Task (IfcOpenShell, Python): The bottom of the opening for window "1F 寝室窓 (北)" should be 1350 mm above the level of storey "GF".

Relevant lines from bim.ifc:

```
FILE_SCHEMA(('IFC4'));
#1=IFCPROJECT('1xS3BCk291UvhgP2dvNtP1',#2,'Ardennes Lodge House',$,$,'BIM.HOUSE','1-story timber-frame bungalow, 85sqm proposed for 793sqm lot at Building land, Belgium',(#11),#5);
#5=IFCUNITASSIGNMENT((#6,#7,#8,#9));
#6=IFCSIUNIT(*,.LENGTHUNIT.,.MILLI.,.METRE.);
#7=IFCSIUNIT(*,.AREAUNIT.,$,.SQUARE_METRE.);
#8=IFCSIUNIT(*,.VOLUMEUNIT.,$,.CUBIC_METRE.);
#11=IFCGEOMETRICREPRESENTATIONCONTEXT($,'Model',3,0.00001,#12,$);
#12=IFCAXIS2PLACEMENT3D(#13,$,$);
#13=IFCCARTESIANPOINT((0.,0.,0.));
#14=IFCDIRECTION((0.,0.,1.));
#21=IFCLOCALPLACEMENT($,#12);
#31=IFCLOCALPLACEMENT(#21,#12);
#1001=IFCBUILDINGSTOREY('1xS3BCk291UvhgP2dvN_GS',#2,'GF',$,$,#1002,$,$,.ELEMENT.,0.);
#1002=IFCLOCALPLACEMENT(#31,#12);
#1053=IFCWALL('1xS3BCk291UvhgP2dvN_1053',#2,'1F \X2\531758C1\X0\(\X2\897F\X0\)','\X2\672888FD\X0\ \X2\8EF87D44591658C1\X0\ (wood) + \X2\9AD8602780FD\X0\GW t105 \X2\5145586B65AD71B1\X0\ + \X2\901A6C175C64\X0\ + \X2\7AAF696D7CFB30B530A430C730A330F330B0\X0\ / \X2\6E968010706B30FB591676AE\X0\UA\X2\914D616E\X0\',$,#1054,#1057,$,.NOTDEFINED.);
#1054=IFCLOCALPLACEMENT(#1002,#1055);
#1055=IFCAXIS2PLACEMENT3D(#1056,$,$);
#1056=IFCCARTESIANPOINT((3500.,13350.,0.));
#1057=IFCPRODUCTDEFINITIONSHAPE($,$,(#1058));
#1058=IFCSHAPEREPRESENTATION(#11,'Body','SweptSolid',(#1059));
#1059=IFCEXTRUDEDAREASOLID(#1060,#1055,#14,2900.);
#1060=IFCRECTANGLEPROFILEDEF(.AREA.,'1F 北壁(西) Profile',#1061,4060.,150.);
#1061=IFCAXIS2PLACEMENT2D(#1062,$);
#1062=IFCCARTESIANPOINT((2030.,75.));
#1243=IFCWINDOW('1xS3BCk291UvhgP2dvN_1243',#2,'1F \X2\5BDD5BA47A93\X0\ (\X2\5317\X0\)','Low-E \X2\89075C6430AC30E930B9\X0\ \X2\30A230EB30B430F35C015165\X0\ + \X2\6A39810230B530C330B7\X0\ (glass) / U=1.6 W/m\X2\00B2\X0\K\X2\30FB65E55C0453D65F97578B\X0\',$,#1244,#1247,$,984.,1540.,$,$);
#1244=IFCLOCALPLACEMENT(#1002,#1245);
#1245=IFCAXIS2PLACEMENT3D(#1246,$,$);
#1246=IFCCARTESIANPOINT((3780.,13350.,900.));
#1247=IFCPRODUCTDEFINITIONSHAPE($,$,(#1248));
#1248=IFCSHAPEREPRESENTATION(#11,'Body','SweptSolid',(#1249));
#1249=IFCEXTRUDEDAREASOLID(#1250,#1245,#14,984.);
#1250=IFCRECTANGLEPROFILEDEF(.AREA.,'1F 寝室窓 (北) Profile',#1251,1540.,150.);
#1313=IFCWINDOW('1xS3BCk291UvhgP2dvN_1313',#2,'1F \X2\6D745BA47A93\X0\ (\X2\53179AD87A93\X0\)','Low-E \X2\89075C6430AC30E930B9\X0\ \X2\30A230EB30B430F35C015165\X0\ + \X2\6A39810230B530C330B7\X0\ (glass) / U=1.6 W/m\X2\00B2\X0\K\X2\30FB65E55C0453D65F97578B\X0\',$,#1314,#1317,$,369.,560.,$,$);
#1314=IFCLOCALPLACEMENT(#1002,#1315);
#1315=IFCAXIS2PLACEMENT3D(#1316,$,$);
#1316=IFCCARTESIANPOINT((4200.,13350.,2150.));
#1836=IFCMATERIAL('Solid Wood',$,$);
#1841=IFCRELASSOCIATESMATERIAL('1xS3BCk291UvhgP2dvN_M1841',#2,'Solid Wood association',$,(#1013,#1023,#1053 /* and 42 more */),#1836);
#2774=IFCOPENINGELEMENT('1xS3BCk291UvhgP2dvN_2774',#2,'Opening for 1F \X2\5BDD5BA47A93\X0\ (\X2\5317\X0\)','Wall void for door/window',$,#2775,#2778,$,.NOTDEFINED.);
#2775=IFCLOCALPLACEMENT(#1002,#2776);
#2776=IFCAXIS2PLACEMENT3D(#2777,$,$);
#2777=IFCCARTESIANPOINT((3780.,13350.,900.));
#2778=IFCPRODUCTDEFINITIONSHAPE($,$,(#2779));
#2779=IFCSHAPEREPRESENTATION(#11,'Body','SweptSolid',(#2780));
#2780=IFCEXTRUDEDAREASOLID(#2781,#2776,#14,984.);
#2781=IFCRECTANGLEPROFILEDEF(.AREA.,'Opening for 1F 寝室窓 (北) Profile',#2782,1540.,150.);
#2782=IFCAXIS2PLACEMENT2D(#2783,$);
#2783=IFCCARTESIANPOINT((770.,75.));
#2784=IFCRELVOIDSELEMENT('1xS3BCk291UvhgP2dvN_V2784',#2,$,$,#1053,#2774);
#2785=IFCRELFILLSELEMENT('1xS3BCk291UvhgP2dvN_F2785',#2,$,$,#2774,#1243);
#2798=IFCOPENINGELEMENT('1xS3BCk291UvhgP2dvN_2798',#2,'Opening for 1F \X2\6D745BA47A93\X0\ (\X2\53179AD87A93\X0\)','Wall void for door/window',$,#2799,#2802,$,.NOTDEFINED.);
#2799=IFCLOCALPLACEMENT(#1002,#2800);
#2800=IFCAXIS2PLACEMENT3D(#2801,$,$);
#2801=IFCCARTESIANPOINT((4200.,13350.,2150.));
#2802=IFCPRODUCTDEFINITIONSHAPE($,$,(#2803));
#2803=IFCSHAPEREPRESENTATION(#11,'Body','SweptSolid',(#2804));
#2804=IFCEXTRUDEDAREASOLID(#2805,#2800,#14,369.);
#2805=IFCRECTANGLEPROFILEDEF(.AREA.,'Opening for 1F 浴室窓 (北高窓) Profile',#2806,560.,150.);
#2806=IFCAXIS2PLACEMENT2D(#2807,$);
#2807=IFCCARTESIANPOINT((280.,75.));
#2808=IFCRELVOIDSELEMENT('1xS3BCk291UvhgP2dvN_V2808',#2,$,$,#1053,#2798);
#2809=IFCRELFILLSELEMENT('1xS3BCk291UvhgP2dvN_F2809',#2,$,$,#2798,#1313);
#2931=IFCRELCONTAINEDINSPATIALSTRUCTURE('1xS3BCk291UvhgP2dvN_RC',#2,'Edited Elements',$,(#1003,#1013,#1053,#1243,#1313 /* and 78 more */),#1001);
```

```python
import numpy as np
import ifcopenshell
import ifcopenshell.api.geometry
import ifcopenshell.geom
import ifcopenshell.util.element
import ifcopenshell.util.placement
import ifcopenshell.util.shape
import ifcopenshell.util.unit

model = ifcopenshell.open("bim.ifc")
unit_scale = ifcopenshell.util.unit.calculate_unit_scale(model)

window = model.by_guid("1xS3BCk291UvhgP2dvN_1243")
opening = window.FillsVoids[0].RelatingOpeningElement
storey = ifcopenshell.util.element.get_container(window, ifc_class="IfcBuildingStorey")
level = ifcopenshell.util.placement.get_local_placement(storey.ObjectPlacement)[2, 3]

# The opening's origin need not be at the sill, so measure its lowest point.
shape = ifcopenshell.geom.create_shape(ifcopenshell.geom.settings(), opening)
bottom = ifcopenshell.util.shape.get_shape_bottom_elevation(shape, shape.geometry) / unit_scale
dz = level + 1.35 / unit_scale - bottom

shift = np.array([0.0, 0.0, dz])
# The window is not placed relative to its opening, so move both.
for product in (opening, window):
    matrix = ifcopenshell.util.placement.get_local_placement(product.ObjectPlacement)
    matrix[:3, 3] += shift
    ifcopenshell.api.geometry.edit_object_placement(model, product=product, matrix=matrix, is_si=False)

print(f"moved by {dz * unit_scale:+.3f} m")

model.write("bim_rev.ifc")
```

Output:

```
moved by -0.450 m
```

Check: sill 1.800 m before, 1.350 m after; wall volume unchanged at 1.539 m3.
